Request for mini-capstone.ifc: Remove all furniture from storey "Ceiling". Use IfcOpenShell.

First a look at what the model holds.

```python
import ifcopenshell
import ifcopenshell.util.element

model = ifcopenshell.open("mini-capstone.ifc")
print(model.schema)
storey = next(s for s in model.by_type("IfcBuildingStorey") if s.Name == "Ceiling")
furniture = [e for e in ifcopenshell.util.element.get_decomposition(storey) if e.is_a("IfcFurnishingElement")]
seen = {}
for e in furniture:
    element_type = ifcopenshell.util.element.get_type(e)
    name = element_type.Name if element_type not in (None, e) else None
    seen[name] = seen.get(name, 0) + 1
for name, count in sorted(seen.items(), key=str):
    print(count, "x", name)
```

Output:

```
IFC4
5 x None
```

```python
import ifcopenshell
import ifcopenshell.api.root
import ifcopenshell.util.element

model = ifcopenshell.open("mini-capstone.ifc")

storey = next(s for s in model.by_type("IfcBuildingStorey") if s.Name == "Ceiling")
furniture = [e for e in ifcopenshell.util.element.get_decomposition(storey) if e.is_a("IfcFurnishingElement")]

for e in furniture:
    ifcopenshell.api.root.remove_product(model, product=e)
print(len(furniture), "removed")

model.write("mini-capstone_v2.ifc")
```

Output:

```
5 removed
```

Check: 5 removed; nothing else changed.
